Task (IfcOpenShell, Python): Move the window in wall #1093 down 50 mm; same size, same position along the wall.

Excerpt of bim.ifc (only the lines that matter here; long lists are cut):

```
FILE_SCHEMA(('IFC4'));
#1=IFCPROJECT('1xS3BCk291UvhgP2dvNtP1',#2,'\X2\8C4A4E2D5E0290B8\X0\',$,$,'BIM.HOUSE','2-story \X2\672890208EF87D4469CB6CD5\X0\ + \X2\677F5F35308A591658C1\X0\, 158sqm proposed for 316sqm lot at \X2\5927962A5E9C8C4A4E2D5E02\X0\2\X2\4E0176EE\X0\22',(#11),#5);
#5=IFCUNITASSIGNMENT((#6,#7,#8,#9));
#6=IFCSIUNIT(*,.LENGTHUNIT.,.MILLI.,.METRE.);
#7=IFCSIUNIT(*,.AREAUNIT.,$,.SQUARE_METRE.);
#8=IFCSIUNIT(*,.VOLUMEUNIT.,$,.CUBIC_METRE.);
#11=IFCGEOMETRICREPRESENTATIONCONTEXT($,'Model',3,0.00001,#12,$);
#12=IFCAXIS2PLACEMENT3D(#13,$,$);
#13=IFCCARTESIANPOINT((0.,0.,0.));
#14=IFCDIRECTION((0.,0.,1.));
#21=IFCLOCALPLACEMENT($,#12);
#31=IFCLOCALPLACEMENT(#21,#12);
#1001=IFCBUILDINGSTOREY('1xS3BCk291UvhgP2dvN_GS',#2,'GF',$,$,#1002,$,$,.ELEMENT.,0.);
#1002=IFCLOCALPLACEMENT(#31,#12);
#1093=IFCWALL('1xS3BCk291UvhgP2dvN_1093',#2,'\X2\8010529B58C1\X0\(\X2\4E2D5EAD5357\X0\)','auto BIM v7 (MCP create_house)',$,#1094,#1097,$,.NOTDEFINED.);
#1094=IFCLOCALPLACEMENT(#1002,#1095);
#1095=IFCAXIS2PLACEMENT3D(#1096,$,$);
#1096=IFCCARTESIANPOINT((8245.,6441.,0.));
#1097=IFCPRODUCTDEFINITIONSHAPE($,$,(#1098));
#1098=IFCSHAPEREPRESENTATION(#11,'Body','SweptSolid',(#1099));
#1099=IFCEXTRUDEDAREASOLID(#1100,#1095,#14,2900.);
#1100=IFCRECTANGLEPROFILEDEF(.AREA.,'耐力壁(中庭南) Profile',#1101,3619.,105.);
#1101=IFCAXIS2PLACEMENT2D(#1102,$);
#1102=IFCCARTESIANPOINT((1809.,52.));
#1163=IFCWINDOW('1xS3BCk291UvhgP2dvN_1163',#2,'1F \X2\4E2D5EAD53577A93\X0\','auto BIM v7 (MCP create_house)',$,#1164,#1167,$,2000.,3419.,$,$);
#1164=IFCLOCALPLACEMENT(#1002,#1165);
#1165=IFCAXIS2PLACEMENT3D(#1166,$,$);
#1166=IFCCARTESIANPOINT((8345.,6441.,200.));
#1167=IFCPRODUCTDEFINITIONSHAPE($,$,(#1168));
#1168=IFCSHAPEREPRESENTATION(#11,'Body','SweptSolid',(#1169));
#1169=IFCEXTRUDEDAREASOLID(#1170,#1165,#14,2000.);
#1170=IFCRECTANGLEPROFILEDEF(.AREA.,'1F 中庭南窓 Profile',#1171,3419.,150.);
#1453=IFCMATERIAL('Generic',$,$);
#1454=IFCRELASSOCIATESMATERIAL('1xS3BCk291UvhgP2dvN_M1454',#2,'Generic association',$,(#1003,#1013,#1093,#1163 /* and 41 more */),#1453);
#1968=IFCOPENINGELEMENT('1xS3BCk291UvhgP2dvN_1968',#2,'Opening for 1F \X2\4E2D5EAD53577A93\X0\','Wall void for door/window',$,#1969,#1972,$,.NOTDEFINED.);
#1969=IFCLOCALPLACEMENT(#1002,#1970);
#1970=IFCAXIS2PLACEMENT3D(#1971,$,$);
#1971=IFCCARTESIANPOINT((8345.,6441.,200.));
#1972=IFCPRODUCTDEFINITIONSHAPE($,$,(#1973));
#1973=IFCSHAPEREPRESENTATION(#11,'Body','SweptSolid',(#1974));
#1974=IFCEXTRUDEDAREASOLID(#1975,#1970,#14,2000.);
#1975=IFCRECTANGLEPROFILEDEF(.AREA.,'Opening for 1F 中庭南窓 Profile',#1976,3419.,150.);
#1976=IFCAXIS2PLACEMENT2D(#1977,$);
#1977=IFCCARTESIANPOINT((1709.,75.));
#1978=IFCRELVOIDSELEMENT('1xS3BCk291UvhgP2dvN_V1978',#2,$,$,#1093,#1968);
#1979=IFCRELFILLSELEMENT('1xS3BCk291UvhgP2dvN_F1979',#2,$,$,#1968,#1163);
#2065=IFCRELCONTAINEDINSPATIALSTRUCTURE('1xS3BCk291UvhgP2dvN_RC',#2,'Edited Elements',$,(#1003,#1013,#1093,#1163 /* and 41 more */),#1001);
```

```python
import numpy as np
import ifcopenshell
import ifcopenshell.api.geometry
import ifcopenshell.util.placement
import ifcopenshell.util.unit

model = ifcopenshell.open("bim.ifc")
unit_scale = ifcopenshell.util.unit.calculate_unit_scale(model)

window = model.by_guid("1xS3BCk291UvhgP2dvN_1163")
opening = window.FillsVoids[0].RelatingOpeningElement
dz = -0.05 / unit_scale

shift = np.array([0.0, 0.0, dz])
# The window is not placed relative to its opening, so move both.
for product in (opening, window):
    matrix = ifcopenshell.util.placement.get_local_placement(product.ObjectPlacement)
    matrix[:3, 3] += shift
    ifcopenshell.api.geometry.edit_object_placement(model, product=product, matrix=matrix, is_si=False)

print(f"moved by {dz * unit_scale:+.3f} m")

model.write("bim_edited.ifc")
```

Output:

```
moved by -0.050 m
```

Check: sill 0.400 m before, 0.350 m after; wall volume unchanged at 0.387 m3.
